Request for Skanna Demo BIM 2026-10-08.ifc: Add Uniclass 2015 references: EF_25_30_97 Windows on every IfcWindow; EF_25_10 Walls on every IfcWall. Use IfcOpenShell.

First a look at what the model holds.

```python
import ifcopenshell

model = ifcopenshell.open("Skanna Demo BIM 2026-10-08.ifc")
print(model.schema)
print("classifications:", [c.Name for c in model.by_type("IfcClassification")])
for ifc_class in ("IfcDoor", "IfcRoof", "IfcStair", "IfcWall", "IfcWindow"):
    print(ifc_class, len(model.by_type(ifc_class)))
```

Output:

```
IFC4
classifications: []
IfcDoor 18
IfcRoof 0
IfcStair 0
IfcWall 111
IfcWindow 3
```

```python
import ifcopenshell
import ifcopenshell.api.classification

model = ifcopenshell.open("Skanna Demo BIM 2026-10-08.ifc")

system = ifcopenshell.api.classification.add_classification(model, classification="Uniclass 2015")

codes = {
    "IfcWindow": ("EF_25_30_97", "Windows"),
    "IfcWall": ("EF_25_10", "Walls"),
}
for ifc_class, (code, name) in codes.items():
    products = model.by_type(ifc_class)
    ifcopenshell.api.classification.add_reference(
        model, products=products, classification=system, identification=code, name=name
    )
    print(code, len(products))

model.write("Skanna Demo BIM 2026-10-08-out.ifc")
```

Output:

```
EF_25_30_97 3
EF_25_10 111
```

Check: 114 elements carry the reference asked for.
